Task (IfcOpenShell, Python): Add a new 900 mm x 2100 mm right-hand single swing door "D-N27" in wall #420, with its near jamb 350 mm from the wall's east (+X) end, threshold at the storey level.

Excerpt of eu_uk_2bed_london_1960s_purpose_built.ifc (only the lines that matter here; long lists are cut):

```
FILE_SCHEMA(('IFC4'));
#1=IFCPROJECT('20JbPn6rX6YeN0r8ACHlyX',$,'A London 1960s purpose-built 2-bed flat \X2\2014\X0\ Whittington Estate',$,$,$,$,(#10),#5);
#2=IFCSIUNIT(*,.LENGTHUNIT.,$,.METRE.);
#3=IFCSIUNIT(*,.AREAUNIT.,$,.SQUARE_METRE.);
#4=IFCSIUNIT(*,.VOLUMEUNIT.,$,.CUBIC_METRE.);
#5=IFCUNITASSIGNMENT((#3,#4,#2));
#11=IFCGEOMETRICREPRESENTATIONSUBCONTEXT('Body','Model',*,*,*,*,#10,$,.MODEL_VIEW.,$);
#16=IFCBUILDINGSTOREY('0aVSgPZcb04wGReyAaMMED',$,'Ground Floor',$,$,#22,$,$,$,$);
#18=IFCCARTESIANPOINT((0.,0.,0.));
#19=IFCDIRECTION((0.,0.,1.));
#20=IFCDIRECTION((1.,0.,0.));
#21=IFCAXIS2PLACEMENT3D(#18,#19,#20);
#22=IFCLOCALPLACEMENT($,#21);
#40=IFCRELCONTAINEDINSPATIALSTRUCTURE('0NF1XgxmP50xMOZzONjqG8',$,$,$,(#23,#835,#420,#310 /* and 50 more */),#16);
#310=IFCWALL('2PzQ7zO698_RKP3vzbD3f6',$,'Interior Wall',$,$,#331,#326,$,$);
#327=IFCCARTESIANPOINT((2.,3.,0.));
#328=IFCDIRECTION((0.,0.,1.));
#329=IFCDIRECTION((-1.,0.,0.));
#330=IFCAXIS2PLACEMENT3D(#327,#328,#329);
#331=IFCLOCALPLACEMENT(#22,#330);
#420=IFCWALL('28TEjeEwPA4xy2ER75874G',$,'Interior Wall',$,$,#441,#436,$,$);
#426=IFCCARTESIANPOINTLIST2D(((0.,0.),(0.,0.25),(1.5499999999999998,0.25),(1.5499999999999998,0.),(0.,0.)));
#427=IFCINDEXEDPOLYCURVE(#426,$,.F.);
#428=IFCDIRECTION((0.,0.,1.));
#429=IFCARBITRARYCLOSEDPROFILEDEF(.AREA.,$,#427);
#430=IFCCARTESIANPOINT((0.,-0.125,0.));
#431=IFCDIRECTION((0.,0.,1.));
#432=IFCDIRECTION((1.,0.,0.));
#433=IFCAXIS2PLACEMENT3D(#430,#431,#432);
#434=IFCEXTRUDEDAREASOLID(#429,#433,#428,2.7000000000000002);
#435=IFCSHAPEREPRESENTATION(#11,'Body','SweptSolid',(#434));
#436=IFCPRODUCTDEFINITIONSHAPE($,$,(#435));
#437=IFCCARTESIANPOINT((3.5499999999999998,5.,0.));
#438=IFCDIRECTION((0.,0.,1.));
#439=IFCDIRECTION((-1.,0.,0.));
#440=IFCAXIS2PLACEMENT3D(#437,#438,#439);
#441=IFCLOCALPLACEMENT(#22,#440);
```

```python
import numpy as np
import ifcopenshell
import ifcopenshell.api.feature
import ifcopenshell.api.geometry
import ifcopenshell.api.root
import ifcopenshell.api.spatial
import ifcopenshell.geom
import ifcopenshell.util.element
import ifcopenshell.util.placement
import ifcopenshell.util.representation
import ifcopenshell.util.shape
import ifcopenshell.util.unit

model = ifcopenshell.open("eu_uk_2bed_london_1960s_purpose_built.ifc")
unit_scale = ifcopenshell.util.unit.calculate_unit_scale(model)
settings = ifcopenshell.geom.settings()


def volume(element):
    """Net volume in cubic metres, openings subtracted."""
    shape = ifcopenshell.geom.create_shape(settings, element)
    return ifcopenshell.util.shape.get_volume(shape.geometry)


wall = model.by_guid("28TEjeEwPA4xy2ER75874G")
storey = ifcopenshell.util.element.get_container(wall, ifc_class="IfcBuildingStorey")
context = ifcopenshell.util.representation.get_context(model, "Model", "Body", "MODEL_VIEW")
before = volume(wall)

width, height, from_end, sill = 0.9, 2.1, 0.35, 0.0  # metres

# The wall runs along its own X axis, and the end named is its -X end.
wall_shape = ifcopenshell.geom.create_shape(settings, wall)
x, y, z = ifcopenshell.util.shape.get_vertices(wall_shape.geometry).T
start = x.min() + from_end
face, thickness = float(y.min()), float(y.max() - y.min())
wall_matrix = ifcopenshell.util.placement.get_local_placement(wall.ObjectPlacement)
level = ifcopenshell.util.placement.get_local_placement(storey.ObjectPlacement)[2, 3]


def in_wall(x, y):
    """Placement at x, y metres in the wall's axes, at sill height."""
    matrix = wall_matrix.copy()
    matrix[:, 3] = wall_matrix @ np.array([x / unit_scale, y / unit_scale, 0.0, 1.0])
    matrix[2, 3] = level + sill / unit_scale
    return matrix


# Opening: a box that overshoots both wall faces by 50 mm.
opening = ifcopenshell.api.root.create_entity(model, ifc_class="IfcOpeningElement", predefined_type="OPENING")
box = ifcopenshell.api.geometry.add_wall_representation(
    model, context=context, length=width, height=height, thickness=thickness + 0.1
)
ifcopenshell.api.geometry.assign_representation(model, product=opening, representation=box)
ifcopenshell.api.geometry.edit_object_placement(model, product=opening, matrix=in_wall(start, face - 0.05), is_si=False)
ifcopenshell.api.feature.add_feature(model, feature=opening, element=wall)

door = ifcopenshell.api.root.create_entity(model, ifc_class="IfcDoor", name="D-N27", predefined_type="DOOR")
door.OverallWidth, door.OverallHeight = width / unit_scale, height / unit_scale
door.OperationType = "SINGLE_SWING_RIGHT"
body = ifcopenshell.api.geometry.add_door_representation(
    model,
    context=context,
    overall_width=door.OverallWidth,
    overall_height=door.OverallHeight,
    operation_type="SINGLE_SWING_RIGHT",
    lining_properties={"LiningDepth": thickness / unit_scale, "ThresholdDepth": thickness / unit_scale},
)
ifcopenshell.api.geometry.assign_representation(model, product=door, representation=body)
ifcopenshell.api.spatial.assign_container(model, products=[door], relating_structure=storey)
ifcopenshell.api.feature.add_filling(model, opening=opening, element=door)

# The lining spans the wall, so the door starts at the wall face.
ifcopenshell.api.geometry.edit_object_placement(model, product=door, matrix=in_wall(start, face), is_si=False)

after = volume(wall)

print(f"wall volume {before:.3f} -> {after:.3f} m3")

model.write("eu_uk_2bed_london_1960s_purpose_built_edited.ifc")
```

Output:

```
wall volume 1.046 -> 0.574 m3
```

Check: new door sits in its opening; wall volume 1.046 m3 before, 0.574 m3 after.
